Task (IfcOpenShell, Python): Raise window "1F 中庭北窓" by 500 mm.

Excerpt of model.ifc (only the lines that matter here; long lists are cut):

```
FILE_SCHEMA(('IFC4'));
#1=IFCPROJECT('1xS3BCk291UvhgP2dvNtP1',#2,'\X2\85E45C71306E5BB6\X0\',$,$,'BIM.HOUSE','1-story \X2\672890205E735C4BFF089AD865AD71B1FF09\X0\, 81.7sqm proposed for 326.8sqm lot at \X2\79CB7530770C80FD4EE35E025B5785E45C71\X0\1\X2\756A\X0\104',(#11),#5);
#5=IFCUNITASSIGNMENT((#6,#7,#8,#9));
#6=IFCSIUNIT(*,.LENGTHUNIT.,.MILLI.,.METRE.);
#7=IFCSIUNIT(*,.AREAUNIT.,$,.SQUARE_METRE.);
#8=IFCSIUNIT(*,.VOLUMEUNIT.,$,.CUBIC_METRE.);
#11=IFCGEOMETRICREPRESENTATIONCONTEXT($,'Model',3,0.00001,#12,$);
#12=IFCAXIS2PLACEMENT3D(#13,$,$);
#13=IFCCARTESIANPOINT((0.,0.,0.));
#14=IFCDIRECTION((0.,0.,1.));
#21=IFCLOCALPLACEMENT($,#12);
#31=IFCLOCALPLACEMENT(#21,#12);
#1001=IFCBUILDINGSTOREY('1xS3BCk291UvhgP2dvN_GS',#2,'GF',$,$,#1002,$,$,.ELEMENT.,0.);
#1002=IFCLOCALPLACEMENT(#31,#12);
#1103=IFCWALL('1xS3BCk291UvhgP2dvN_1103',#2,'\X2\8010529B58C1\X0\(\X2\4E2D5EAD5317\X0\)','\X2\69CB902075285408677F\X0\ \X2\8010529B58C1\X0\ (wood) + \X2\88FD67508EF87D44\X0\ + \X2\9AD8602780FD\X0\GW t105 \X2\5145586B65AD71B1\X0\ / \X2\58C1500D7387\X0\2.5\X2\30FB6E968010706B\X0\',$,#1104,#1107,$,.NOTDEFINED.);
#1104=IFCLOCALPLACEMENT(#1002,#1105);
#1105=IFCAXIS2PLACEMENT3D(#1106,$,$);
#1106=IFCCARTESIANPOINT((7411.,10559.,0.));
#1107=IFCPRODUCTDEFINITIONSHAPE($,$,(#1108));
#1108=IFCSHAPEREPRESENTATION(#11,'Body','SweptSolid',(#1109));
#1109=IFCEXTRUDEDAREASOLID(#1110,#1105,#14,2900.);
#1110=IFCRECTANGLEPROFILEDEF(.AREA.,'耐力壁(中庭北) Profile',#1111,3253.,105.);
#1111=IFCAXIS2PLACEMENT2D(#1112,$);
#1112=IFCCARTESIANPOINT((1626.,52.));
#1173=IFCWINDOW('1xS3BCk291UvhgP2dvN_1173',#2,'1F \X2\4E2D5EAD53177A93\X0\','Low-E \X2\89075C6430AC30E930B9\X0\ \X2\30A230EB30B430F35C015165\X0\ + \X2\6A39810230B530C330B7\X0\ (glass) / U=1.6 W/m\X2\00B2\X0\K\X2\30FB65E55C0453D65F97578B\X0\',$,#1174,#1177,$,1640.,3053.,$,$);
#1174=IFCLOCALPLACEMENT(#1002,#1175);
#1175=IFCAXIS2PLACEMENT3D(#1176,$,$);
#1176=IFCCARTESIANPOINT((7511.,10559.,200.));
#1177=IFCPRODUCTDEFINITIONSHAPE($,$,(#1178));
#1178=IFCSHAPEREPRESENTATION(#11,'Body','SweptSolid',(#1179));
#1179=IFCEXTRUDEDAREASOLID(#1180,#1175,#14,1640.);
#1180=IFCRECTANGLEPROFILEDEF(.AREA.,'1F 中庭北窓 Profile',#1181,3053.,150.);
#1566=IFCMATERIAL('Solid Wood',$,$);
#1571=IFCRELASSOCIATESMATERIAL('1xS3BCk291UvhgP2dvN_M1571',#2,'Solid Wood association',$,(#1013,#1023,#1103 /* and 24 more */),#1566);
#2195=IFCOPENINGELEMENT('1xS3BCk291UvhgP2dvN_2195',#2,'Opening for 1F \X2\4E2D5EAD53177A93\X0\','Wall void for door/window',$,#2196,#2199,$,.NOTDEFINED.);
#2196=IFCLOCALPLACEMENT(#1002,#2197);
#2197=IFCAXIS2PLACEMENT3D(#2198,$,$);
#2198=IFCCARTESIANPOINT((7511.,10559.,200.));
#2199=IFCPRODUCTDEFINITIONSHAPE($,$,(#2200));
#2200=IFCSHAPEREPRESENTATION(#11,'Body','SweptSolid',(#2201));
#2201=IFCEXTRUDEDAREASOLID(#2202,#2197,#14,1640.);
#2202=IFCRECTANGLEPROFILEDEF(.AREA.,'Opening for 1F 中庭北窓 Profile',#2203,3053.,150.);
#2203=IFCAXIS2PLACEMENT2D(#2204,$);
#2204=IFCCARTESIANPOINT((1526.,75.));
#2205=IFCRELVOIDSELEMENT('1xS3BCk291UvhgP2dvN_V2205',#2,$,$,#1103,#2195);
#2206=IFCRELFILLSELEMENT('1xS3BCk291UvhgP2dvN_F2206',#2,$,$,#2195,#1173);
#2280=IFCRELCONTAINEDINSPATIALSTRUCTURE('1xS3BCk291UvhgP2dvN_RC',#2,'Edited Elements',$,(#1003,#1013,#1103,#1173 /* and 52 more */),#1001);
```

```python
import numpy as np
import ifcopenshell
import ifcopenshell.api.geometry
import ifcopenshell.util.placement
import ifcopenshell.util.unit

model = ifcopenshell.open("model.ifc")
unit_scale = ifcopenshell.util.unit.calculate_unit_scale(model)

window = model.by_guid("1xS3BCk291UvhgP2dvN_1173")
opening = window.FillsVoids[0].RelatingOpeningElement
dz = 500.0

shift = np.array([0.0, 0.0, dz])
# The window is not placed relative to its opening, so move both.
for product in (opening, window):
    matrix = ifcopenshell.util.placement.get_local_placement(product.ObjectPlacement)
    matrix[:3, 3] += shift
    ifcopenshell.api.geometry.edit_object_placement(model, product=product, matrix=matrix, is_si=False)

print(f"moved by {dz * unit_scale:+.3f} m")

model.write("model_edited.ifc")
```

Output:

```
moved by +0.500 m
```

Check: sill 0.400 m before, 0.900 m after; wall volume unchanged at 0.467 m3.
